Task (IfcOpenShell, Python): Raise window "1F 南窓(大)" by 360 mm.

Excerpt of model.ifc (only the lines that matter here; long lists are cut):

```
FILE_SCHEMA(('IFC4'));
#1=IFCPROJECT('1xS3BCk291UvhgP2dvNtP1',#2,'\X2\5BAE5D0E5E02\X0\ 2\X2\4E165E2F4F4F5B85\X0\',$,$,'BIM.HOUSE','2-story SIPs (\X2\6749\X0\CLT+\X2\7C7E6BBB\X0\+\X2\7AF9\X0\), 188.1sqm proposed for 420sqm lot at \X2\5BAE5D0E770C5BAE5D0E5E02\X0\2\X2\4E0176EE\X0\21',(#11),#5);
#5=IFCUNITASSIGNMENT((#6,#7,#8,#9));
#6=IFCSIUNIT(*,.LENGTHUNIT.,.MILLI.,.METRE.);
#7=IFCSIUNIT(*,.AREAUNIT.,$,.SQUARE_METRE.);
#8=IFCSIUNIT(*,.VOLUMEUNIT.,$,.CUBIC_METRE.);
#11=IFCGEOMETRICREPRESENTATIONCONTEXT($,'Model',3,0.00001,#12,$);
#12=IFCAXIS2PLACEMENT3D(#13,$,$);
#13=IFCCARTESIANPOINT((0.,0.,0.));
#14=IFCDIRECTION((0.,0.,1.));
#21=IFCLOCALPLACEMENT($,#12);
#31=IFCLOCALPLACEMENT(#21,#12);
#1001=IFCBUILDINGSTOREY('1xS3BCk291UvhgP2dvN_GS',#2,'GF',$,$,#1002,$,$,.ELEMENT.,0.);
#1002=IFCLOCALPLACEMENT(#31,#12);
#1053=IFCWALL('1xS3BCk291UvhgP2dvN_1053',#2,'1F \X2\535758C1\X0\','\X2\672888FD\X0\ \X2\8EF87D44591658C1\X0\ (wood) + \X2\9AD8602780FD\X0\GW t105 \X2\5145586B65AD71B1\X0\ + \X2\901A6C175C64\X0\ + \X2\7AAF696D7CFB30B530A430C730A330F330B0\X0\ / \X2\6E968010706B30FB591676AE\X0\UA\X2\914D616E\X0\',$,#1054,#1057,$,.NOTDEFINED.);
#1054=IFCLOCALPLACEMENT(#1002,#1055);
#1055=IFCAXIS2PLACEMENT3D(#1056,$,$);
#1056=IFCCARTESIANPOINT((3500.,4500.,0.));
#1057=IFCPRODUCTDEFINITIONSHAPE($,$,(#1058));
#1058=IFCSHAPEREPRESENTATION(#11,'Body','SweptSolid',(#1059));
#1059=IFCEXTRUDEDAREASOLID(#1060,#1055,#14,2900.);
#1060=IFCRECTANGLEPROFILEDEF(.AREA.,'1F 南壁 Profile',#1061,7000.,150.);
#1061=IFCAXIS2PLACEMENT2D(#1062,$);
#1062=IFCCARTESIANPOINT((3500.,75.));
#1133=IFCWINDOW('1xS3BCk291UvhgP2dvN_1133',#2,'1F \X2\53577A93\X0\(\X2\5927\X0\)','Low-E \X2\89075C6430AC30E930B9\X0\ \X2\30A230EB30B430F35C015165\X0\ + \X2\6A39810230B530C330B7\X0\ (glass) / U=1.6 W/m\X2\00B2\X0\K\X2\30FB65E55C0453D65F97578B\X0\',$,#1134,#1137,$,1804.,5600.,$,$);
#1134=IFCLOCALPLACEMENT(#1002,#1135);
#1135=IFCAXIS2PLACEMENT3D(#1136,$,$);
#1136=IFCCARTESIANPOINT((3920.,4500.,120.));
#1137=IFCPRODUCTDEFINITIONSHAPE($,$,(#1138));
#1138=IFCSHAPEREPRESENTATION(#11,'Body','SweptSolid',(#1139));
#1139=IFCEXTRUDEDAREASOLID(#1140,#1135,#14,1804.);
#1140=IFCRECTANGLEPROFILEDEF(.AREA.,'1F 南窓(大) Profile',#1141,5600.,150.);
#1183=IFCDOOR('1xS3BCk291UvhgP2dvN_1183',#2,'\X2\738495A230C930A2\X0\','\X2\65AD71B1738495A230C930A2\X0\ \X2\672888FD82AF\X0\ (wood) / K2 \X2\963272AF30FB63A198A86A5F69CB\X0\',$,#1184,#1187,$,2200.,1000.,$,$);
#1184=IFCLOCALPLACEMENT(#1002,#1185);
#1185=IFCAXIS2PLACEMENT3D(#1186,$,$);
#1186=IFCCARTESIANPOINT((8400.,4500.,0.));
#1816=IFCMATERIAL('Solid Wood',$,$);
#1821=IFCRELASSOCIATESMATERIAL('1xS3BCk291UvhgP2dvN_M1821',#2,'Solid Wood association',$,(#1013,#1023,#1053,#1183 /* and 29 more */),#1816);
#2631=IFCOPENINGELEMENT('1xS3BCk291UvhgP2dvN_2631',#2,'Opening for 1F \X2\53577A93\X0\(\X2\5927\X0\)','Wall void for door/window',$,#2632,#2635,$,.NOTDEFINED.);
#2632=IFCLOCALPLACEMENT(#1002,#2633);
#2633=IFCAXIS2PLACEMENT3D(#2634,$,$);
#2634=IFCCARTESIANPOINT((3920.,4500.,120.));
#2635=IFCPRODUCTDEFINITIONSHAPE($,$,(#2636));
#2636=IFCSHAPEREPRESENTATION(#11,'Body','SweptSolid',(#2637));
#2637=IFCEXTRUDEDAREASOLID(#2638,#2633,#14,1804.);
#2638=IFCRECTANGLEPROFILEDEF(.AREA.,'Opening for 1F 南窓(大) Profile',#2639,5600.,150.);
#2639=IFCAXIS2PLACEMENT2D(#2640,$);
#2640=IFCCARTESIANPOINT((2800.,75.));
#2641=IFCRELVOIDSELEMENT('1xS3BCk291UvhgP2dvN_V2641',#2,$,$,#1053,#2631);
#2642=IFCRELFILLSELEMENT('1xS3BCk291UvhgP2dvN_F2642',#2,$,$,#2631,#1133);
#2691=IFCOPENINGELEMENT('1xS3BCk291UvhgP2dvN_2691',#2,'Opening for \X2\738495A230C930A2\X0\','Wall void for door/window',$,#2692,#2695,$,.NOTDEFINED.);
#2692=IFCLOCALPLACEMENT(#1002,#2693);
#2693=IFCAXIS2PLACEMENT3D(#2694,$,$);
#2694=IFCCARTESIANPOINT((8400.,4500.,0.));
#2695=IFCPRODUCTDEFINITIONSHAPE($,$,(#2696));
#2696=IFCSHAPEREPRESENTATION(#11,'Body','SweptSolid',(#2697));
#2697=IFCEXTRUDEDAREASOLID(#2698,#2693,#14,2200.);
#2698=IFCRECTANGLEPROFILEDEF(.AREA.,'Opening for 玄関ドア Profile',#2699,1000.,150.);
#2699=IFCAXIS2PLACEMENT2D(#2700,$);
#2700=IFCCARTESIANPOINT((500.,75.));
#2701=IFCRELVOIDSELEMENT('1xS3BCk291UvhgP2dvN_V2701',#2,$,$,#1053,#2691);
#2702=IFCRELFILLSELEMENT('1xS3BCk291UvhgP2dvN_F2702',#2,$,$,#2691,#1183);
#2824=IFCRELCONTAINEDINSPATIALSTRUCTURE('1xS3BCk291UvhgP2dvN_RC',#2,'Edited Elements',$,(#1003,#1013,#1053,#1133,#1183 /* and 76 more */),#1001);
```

```python
import numpy as np
import ifcopenshell
import ifcopenshell.api.geometry
import ifcopenshell.util.placement
import ifcopenshell.util.unit

model = ifcopenshell.open("model.ifc")
unit_scale = ifcopenshell.util.unit.calculate_unit_scale(model)

window = model.by_guid("1xS3BCk291UvhgP2dvN_1133")
opening = window.FillsVoids[0].RelatingOpeningElement
dz = 0.36 / unit_scale

shift = np.array([0.0, 0.0, dz])
# The window is not placed relative to its opening, so move both.
for product in (opening, window):
    matrix = ifcopenshell.util.placement.get_local_placement(product.ObjectPlacement)
    matrix[:3, 3] += shift
    ifcopenshell.api.geometry.edit_object_placement(model, product=product, matrix=matrix, is_si=False)

print(f"moved by {dz * unit_scale:+.3f} m")

model.write("model-out.ifc")
```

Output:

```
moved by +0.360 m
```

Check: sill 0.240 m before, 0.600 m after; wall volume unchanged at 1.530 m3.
